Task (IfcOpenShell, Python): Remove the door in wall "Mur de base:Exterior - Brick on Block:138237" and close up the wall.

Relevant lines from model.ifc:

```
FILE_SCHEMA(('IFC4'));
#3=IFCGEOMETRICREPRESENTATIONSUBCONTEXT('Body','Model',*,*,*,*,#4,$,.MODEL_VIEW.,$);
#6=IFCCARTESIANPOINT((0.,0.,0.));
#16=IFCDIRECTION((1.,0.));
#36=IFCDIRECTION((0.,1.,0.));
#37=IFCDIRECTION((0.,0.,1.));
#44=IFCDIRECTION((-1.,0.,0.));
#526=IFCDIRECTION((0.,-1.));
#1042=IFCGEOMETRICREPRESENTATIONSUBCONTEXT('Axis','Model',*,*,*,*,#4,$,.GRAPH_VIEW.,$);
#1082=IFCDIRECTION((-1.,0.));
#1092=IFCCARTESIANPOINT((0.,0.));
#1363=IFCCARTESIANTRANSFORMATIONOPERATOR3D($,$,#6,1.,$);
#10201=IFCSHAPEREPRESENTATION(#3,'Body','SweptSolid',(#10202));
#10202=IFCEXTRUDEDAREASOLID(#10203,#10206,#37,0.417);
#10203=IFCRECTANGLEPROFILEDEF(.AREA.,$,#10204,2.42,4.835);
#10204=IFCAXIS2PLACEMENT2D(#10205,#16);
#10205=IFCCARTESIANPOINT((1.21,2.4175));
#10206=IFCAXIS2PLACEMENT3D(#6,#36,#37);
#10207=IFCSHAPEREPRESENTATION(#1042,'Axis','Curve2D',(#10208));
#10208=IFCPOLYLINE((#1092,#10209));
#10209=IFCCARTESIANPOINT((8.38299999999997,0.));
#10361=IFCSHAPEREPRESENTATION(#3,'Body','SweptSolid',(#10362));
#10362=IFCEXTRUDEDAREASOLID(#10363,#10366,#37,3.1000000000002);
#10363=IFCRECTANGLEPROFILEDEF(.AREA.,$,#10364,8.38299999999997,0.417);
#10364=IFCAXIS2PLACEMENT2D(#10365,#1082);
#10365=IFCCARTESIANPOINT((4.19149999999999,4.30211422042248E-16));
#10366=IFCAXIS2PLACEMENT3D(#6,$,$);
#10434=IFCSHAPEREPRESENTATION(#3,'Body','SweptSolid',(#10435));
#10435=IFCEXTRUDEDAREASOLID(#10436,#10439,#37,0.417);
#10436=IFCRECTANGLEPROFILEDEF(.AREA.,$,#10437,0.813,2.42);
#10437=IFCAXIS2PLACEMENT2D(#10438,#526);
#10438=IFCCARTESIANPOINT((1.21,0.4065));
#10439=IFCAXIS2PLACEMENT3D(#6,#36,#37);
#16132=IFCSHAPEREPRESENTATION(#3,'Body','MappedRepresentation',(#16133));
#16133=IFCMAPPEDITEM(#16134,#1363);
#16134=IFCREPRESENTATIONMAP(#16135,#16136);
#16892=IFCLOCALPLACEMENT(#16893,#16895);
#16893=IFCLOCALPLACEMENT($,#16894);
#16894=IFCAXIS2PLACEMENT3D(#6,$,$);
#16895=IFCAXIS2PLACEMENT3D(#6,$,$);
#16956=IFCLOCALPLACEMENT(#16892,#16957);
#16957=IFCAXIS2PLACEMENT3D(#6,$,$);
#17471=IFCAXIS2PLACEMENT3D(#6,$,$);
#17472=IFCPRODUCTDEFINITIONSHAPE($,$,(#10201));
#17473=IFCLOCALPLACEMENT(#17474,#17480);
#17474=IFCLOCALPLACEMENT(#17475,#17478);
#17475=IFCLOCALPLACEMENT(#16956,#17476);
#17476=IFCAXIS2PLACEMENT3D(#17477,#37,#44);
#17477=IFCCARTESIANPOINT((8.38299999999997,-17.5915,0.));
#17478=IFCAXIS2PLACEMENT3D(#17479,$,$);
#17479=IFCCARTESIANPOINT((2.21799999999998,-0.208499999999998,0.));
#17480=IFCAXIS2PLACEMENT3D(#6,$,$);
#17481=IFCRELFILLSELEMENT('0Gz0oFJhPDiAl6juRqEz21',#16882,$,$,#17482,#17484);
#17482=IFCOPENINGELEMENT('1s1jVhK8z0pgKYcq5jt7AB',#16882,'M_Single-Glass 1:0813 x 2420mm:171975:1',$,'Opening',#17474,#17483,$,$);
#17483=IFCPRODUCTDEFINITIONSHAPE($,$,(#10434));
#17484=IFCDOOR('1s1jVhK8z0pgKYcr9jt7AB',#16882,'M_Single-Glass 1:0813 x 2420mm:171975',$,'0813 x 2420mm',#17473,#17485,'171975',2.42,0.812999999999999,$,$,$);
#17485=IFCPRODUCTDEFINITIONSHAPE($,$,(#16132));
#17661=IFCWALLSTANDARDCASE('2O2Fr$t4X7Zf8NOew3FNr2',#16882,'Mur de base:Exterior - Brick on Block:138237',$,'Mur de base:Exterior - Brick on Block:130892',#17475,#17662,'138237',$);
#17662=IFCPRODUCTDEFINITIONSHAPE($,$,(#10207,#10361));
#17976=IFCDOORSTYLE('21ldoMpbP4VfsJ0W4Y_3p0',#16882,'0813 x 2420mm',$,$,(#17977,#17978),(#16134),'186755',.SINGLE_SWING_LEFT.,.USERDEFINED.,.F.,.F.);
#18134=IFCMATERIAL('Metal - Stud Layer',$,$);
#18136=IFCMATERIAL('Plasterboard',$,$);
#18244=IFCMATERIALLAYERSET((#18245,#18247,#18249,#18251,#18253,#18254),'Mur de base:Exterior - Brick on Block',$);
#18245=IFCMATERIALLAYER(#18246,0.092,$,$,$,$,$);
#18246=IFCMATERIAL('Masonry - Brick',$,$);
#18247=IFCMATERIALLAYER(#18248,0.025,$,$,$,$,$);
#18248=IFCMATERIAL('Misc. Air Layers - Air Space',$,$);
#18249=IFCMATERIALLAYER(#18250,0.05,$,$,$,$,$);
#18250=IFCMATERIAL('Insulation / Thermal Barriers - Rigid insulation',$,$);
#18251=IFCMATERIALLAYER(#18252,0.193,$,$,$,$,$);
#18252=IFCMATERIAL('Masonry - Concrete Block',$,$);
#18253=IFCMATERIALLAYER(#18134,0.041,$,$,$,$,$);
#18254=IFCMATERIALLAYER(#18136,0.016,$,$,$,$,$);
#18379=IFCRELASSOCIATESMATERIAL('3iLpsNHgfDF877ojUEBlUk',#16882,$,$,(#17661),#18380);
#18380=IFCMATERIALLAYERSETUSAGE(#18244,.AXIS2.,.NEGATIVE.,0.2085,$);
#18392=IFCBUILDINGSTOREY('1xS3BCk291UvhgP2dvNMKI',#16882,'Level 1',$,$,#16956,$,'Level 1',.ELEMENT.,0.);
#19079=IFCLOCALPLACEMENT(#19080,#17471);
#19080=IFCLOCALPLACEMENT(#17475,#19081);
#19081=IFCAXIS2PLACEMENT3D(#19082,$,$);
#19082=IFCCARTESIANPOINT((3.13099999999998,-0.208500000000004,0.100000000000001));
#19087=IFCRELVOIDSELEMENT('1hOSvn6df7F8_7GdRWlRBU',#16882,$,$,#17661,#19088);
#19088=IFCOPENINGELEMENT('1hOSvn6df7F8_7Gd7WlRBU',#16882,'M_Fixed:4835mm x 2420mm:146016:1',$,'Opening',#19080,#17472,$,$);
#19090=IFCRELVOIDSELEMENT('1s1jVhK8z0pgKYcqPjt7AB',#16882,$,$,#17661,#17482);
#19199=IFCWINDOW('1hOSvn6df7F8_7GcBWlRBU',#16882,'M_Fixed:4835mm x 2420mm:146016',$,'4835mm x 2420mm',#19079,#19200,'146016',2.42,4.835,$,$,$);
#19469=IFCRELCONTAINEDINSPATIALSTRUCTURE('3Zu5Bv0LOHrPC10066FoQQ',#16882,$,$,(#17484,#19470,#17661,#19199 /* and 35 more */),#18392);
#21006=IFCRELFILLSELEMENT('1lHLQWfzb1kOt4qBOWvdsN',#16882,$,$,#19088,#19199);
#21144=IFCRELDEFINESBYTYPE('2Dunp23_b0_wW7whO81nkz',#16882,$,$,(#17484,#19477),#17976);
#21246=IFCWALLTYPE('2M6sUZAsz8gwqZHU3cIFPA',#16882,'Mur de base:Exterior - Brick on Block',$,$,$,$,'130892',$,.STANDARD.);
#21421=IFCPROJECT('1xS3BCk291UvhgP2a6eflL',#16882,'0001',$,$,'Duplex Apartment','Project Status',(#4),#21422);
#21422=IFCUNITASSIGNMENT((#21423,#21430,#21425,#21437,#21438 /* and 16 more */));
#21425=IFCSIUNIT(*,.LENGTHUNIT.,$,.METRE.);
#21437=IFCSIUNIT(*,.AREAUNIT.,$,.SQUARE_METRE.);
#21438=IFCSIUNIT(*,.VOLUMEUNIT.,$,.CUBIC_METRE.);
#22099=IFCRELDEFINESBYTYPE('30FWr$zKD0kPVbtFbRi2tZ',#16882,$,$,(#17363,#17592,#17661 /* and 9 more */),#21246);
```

```python
import ifcopenshell
import ifcopenshell.api.feature
import ifcopenshell.api.root
import ifcopenshell.geom
import ifcopenshell.util.shape

model = ifcopenshell.open("model.ifc")
settings = ifcopenshell.geom.settings()


def volume(element):
    """Net volume in cubic metres, openings subtracted."""
    shape = ifcopenshell.geom.create_shape(settings, element)
    return ifcopenshell.util.shape.get_volume(shape.geometry)


door = model.by_guid("1s1jVhK8z0pgKYcr9jt7AB")
opening = door.FillsVoids[0].RelatingOpeningElement
wall = opening.VoidsElements[0].RelatingBuildingElement
before = volume(wall)

ifcopenshell.api.root.remove_product(model, product=door)
ifcopenshell.api.feature.remove_feature(model, feature=opening)

after = volume(wall)

print(f"wall volume {before:.3f} -> {after:.3f} m3")

model.write("model_v2.ifc")
```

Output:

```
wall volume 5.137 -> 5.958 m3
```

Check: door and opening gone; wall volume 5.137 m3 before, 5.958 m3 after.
